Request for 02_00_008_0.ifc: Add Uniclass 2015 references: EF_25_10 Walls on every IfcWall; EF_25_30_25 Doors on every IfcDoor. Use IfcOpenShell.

First a look at what the model holds.

```python
import ifcopenshell

model = ifcopenshell.open("02_00_008_0.ifc")
print(model.schema)
print("classifications:", [c.Name for c in model.by_type("IfcClassification")])
for ifc_class in ("IfcDoor", "IfcRoof", "IfcStair", "IfcWall", "IfcWindow"):
    print(ifc_class, len(model.by_type(ifc_class)))
```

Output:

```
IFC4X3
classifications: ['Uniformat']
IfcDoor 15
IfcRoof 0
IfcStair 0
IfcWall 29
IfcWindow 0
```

```python
import ifcopenshell
import ifcopenshell.api.classification

model = ifcopenshell.open("02_00_008_0.ifc")

system = ifcopenshell.api.classification.add_classification(model, classification="Uniclass 2015")

codes = {
    "IfcWall": ("EF_25_10", "Walls"),
    "IfcDoor": ("EF_25_30_25", "Doors"),
}
for ifc_class, (code, name) in codes.items():
    products = model.by_type(ifc_class)
    ifcopenshell.api.classification.add_reference(
        model, products=products, classification=system, identification=code, name=name
    )
    print(code, len(products))

model.write("02_00_008_0_v2.ifc")
```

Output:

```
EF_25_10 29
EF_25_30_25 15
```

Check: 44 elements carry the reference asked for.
